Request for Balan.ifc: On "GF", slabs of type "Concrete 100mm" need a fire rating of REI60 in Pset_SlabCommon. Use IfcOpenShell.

First a look at what the model holds.

```python
import ifcopenshell
import ifcopenshell.util.element

model = ifcopenshell.open("Balan.ifc")
print(model.schema)
storey = next(s for s in model.by_type("IfcBuildingStorey") if s.Name == "GF")
slabs = [e for e in ifcopenshell.util.element.get_decomposition(storey) if e.is_a("IfcSlab")]
seen = {}
for e in slabs:
    element_type = ifcopenshell.util.element.get_type(e)
    key = (element_type.Name if element_type != e and element_type else None, ifcopenshell.util.element.get_pset(e, "Pset_SlabCommon", "FireRating"))
    seen[key] = seen.get(key, 0) + 1
for (name, value), count in sorted(seen.items(), key=str):
    print(count, "x", name, "|", value)
```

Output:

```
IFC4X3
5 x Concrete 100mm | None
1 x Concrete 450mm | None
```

```python
import ifcopenshell
import ifcopenshell.api.pset
import ifcopenshell.util.element

model = ifcopenshell.open("Balan.ifc")

storey = next(s for s in model.by_type("IfcBuildingStorey") if s.Name == "GF")
slabs = [e for e in ifcopenshell.util.element.get_decomposition(storey) if e.is_a("IfcSlab")]

count = 0
for e in slabs:
    element_type = ifcopenshell.util.element.get_type(e)
    if element_type in (None, e) or element_type.Name != "Concrete 100mm":
        continue
    # add_pset returns the element's existing set when there is one.
    pset = ifcopenshell.api.pset.add_pset(model, product=e, name="Pset_SlabCommon")
    ifcopenshell.api.pset.edit_pset(model, pset=pset, properties={"FireRating": "REI60"})
    count += 1

print(count, "slabs updated")

model.write("Balan_v2.ifc")
```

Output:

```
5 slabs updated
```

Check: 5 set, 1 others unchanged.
